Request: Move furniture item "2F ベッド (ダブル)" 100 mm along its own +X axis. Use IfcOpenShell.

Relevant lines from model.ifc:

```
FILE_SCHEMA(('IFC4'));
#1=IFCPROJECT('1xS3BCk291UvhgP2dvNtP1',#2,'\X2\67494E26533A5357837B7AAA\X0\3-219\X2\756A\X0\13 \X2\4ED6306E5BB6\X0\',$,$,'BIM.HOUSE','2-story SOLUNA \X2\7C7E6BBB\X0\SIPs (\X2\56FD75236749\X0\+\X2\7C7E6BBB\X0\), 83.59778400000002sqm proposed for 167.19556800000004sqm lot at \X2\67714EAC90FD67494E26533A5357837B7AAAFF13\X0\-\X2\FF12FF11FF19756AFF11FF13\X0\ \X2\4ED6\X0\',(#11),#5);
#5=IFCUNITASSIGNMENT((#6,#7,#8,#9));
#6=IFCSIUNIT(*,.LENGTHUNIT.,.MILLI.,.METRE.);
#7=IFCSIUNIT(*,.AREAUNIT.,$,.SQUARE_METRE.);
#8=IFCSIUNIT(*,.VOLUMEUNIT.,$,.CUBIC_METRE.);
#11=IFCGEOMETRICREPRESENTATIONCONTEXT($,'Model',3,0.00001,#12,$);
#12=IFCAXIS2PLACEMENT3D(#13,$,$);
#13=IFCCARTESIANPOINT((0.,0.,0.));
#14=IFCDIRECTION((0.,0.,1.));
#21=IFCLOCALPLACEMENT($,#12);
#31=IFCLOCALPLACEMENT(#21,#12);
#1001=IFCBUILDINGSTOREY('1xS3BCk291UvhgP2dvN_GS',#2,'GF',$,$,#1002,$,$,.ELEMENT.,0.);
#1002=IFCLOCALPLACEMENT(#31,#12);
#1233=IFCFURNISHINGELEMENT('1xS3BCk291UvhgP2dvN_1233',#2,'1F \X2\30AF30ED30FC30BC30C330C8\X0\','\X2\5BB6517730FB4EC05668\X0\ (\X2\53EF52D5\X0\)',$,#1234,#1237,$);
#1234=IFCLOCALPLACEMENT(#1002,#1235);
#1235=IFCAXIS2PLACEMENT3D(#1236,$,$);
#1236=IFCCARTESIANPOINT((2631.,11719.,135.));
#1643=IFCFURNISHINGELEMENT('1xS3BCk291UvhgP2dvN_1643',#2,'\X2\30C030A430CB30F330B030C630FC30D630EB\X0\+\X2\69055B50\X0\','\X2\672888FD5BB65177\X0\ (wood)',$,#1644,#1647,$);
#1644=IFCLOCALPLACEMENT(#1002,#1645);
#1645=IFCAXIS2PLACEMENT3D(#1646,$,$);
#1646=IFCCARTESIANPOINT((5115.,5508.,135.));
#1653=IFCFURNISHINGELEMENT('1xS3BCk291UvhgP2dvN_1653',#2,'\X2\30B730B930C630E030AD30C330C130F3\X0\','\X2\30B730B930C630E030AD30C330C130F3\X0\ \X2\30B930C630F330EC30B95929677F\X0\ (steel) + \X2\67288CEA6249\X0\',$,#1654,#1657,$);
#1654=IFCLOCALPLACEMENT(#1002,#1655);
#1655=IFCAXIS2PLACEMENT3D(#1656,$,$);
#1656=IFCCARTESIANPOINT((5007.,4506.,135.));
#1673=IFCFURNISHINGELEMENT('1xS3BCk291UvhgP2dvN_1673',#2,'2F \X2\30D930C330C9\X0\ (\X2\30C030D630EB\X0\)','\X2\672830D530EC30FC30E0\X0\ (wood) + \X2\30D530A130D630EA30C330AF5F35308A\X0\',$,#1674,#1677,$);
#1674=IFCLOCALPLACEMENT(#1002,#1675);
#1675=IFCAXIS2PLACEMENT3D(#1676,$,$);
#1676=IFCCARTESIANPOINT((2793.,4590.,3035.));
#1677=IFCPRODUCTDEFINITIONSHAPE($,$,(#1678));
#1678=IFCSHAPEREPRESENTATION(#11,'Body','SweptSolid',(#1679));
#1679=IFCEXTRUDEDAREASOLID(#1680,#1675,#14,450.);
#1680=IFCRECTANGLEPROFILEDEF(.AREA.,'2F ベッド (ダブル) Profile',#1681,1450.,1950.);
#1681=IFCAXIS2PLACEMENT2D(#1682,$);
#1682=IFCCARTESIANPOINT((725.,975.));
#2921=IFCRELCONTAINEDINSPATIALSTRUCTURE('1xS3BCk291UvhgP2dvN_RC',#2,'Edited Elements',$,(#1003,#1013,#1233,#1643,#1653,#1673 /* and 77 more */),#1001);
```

```python
import ifcopenshell
import ifcopenshell.api.geometry
import ifcopenshell.util.placement

model = ifcopenshell.open("model.ifc")

item = model.by_guid("1xS3BCk291UvhgP2dvN_1673")
matrix = ifcopenshell.util.placement.get_local_placement(item.ObjectPlacement)
matrix[:3, 3] += matrix[:3, 0] * 100.0
ifcopenshell.api.geometry.edit_object_placement(model, product=item, matrix=matrix, is_si=False)

print(ifcopenshell.util.placement.get_local_placement(item.ObjectPlacement).round(3) + 0.0)

model.write("model_rev.ifc")
```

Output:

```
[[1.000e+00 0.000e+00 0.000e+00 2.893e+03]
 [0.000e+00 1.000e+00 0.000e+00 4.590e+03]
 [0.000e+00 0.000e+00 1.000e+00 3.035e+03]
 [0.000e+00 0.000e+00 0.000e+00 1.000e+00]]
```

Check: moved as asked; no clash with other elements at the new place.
